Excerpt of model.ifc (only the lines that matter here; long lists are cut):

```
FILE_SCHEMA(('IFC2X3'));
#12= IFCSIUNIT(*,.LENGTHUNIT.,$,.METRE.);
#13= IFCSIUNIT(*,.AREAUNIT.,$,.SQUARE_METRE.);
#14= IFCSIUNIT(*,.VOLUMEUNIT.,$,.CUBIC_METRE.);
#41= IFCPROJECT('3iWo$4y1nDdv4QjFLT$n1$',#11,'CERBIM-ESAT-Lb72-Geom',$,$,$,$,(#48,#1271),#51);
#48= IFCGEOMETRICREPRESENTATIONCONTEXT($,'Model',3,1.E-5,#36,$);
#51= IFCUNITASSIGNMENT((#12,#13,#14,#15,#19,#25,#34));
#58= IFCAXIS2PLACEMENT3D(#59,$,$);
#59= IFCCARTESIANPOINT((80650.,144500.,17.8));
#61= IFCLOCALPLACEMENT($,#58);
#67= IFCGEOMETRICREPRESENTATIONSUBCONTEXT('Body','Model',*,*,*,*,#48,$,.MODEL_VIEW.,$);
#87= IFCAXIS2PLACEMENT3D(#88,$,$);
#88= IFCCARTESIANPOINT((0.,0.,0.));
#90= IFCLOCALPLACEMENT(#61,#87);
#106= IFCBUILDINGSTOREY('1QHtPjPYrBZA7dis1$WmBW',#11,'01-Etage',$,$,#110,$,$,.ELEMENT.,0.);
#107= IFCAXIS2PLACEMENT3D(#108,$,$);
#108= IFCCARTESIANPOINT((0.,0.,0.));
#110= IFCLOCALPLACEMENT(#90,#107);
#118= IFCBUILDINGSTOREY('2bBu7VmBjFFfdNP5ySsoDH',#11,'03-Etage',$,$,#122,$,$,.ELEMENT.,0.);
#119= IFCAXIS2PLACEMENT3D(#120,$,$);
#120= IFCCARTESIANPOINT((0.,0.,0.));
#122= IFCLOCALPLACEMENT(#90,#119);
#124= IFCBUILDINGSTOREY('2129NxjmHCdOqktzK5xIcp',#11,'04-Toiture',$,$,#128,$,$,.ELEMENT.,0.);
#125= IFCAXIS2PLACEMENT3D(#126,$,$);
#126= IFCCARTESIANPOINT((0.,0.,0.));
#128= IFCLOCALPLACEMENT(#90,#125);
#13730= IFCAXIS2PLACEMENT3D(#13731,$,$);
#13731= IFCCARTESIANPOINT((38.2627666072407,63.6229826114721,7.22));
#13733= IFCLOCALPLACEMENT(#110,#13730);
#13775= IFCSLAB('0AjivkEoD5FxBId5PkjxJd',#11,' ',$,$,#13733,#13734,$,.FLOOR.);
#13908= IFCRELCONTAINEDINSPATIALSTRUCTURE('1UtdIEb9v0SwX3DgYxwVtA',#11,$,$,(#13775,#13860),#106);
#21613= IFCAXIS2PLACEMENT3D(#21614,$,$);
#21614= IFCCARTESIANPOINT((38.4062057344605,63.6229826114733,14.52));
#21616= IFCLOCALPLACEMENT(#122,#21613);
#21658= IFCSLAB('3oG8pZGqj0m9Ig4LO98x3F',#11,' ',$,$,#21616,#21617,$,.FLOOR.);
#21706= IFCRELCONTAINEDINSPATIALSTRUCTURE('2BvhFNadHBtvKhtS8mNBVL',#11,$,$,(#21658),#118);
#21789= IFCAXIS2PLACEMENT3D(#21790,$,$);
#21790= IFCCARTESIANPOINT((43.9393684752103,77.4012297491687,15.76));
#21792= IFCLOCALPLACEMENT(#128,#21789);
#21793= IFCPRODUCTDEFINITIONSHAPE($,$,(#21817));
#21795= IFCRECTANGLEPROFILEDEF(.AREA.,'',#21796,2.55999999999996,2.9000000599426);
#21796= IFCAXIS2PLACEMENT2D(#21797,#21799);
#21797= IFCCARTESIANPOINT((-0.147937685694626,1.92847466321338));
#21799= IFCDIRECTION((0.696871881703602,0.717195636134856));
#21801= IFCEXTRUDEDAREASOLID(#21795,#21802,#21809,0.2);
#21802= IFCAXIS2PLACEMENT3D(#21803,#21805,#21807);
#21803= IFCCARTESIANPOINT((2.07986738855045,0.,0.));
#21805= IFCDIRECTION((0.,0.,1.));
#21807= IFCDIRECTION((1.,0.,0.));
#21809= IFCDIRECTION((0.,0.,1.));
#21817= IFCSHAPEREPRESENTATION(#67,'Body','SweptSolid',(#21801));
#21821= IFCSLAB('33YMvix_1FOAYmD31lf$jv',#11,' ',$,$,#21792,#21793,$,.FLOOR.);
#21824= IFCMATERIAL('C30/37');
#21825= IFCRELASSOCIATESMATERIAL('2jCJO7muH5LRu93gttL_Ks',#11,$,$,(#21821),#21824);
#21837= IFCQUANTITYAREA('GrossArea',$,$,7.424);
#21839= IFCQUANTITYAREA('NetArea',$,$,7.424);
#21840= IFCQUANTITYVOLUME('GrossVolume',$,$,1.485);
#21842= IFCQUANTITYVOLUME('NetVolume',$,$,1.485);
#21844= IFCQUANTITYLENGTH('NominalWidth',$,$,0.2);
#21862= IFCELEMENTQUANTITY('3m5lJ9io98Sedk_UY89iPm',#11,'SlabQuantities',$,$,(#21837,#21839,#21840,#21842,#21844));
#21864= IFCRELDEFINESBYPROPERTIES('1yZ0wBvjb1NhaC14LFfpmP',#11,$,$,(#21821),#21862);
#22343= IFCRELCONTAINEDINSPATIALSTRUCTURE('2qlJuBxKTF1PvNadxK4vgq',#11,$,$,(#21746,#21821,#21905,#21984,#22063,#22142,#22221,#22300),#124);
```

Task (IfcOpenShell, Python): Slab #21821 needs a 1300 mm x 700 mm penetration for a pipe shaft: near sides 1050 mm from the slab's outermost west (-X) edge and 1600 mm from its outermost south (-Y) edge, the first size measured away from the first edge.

```python
import numpy as np
import ifcopenshell
import ifcopenshell.api.feature
import ifcopenshell.api.geometry
import ifcopenshell.api.pset
import ifcopenshell.api.root
import ifcopenshell.geom
import ifcopenshell.util.element
import ifcopenshell.util.placement
import ifcopenshell.util.representation
import ifcopenshell.util.shape
import ifcopenshell.util.unit

model = ifcopenshell.open("model.ifc")
unit_scale = ifcopenshell.util.unit.calculate_unit_scale(model)
area_scale = ifcopenshell.util.unit.calculate_unit_scale(model, "AREAUNIT")
volume_scale = ifcopenshell.util.unit.calculate_unit_scale(model, "VOLUMEUNIT")
settings = ifcopenshell.geom.settings()


def volume(element):
    """Net volume in cubic metres, openings subtracted."""
    shape = ifcopenshell.geom.create_shape(settings, element)
    return ifcopenshell.util.shape.get_volume(shape.geometry)


slab = model.by_guid("33YMvix_1FOAYmD31lf$jv")
before = volume(slab)

# Extent in the slab's own axes, in metres. The edges named are its -X and -Y sides.
slab_shape = ifcopenshell.geom.create_shape(settings, slab)
vertices = ifcopenshell.util.shape.get_vertices(slab_shape.geometry)
x_min, y_min, bottom = vertices.min(axis=0)
top = vertices[:, 2].max()

opening = ifcopenshell.api.root.create_entity(model, ifc_class="IfcOpeningElement", name="Pipe shaft opening")
context = ifcopenshell.util.representation.get_context(model, "Model", "Body", "MODEL_VIEW")
width, depth = 1.3, 0.7
outline = [(0.0, 0.0), (width, 0.0), (width, depth), (0.0, depth), (0.0, 0.0)]
# Overshoot both faces by 50 mm so the cut is clean.
shape = ifcopenshell.api.geometry.add_slab_representation(
    model, context=context, depth=top - bottom + 0.1, polyline=outline
)
ifcopenshell.api.geometry.assign_representation(model, product=opening, representation=shape)

matrix = ifcopenshell.util.placement.get_local_placement(slab.ObjectPlacement)
matrix[:, 3] = matrix @ np.append(np.array([x_min + 1.05, y_min + 1.6, bottom - 0.05]) / unit_scale, 1.0)
ifcopenshell.api.geometry.edit_object_placement(model, product=opening, matrix=matrix, is_si=False)
ifcopenshell.api.feature.add_feature(model, feature=opening, element=slab)

after = volume(slab)

# Update the slab's stored quantities.
qto = model.by_id(ifcopenshell.util.element.get_pset(slab, "SlabQuantities", should_inherit=False)["id"])
ifcopenshell.api.pset.edit_qto(model, qto=qto, properties={
    "NetArea": after / (top - bottom) / area_scale,
    "NetVolume": after / volume_scale,
})

print(f"slab volume {before:.3f} -> {after:.3f} m3")

model.write("model_updated.ifc")
```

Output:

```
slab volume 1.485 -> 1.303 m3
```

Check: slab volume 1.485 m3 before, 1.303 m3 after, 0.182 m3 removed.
